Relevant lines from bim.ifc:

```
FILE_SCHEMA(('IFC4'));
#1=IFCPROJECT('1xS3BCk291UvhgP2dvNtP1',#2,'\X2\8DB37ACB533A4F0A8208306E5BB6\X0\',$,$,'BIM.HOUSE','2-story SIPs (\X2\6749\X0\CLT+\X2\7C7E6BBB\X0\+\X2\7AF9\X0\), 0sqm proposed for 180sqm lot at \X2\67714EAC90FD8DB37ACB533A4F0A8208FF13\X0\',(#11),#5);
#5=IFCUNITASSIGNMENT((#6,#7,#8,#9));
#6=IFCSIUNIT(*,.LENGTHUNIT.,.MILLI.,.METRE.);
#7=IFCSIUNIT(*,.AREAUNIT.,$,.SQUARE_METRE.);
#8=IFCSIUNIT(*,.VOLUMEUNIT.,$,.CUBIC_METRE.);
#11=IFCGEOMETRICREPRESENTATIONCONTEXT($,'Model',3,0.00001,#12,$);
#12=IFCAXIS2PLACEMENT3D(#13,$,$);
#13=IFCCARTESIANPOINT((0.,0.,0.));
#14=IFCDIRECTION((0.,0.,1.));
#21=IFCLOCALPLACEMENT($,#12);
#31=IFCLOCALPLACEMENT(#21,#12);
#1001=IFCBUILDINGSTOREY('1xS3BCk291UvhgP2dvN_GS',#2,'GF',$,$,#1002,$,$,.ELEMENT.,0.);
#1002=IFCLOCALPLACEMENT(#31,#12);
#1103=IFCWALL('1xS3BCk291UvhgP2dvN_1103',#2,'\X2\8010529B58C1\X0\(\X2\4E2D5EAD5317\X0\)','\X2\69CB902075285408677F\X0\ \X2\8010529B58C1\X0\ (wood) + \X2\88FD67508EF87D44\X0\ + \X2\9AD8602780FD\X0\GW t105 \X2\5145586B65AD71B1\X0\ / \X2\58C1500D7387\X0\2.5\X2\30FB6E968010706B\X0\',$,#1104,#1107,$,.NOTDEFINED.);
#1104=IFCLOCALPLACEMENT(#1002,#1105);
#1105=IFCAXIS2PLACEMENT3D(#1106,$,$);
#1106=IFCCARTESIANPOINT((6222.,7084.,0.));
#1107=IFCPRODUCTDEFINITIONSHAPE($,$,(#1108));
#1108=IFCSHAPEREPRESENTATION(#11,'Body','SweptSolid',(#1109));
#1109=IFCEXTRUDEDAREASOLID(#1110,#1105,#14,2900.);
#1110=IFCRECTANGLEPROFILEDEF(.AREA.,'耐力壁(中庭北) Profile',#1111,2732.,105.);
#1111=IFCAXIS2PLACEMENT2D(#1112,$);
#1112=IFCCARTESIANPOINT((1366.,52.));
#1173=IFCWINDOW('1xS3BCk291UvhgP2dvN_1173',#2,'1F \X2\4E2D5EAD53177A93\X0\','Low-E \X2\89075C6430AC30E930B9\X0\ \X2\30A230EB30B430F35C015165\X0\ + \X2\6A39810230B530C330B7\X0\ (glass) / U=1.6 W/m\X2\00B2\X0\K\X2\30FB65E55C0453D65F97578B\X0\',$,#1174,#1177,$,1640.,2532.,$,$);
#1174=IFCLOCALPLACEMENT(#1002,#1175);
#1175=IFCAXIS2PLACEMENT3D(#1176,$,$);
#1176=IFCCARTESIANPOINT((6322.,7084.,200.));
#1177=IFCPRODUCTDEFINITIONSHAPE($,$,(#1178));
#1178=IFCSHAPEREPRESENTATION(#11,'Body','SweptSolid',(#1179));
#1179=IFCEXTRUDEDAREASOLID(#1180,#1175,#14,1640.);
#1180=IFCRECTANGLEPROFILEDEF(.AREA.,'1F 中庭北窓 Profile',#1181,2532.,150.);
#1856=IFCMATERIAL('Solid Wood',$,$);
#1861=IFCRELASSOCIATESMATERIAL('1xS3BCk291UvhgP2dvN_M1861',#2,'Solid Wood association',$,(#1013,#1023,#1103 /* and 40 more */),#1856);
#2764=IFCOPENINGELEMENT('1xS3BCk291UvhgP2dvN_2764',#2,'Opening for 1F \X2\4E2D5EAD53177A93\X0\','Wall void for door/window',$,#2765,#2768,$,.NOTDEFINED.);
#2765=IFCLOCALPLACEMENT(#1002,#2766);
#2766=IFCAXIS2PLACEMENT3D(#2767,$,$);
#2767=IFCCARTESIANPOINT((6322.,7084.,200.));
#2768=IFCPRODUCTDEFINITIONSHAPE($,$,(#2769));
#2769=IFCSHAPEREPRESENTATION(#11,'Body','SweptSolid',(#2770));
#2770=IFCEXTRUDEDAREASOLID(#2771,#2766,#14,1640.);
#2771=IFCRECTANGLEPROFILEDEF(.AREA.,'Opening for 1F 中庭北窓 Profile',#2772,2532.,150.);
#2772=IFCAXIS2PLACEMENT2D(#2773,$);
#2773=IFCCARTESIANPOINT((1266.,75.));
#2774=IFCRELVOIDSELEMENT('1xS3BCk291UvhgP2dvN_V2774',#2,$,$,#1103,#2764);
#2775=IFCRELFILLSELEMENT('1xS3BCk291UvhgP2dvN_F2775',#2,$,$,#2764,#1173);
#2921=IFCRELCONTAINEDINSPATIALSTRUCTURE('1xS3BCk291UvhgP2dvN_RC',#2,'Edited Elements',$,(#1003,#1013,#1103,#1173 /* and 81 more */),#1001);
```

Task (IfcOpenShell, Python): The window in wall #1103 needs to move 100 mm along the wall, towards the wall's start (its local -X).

```python
import ifcopenshell
import ifcopenshell.api.geometry
import ifcopenshell.util.placement

model = ifcopenshell.open("bim.ifc")

window = model.by_guid("1xS3BCk291UvhgP2dvN_1173")
opening = window.FillsVoids[0].RelatingOpeningElement
wall = opening.VoidsElements[0].RelatingBuildingElement

wall_matrix = ifcopenshell.util.placement.get_local_placement(wall.ObjectPlacement)
shift = wall_matrix[:3, 0] * -100.0
before = ifcopenshell.util.placement.get_local_placement(window.ObjectPlacement)[:3, 3].copy()

# The window is not placed relative to its opening, so move both.
for product in (opening, window):
    matrix = ifcopenshell.util.placement.get_local_placement(product.ObjectPlacement)
    matrix[:3, 3] += shift
    ifcopenshell.api.geometry.edit_object_placement(model, product=product, matrix=matrix, is_si=False)

after = ifcopenshell.util.placement.get_local_placement(window.ObjectPlacement)[:3, 3]
print("window moved by", (after - before).round(3) + 0.0)

model.write("bim_updated.ifc")
```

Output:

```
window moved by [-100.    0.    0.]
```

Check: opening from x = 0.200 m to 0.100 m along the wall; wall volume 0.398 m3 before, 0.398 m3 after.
